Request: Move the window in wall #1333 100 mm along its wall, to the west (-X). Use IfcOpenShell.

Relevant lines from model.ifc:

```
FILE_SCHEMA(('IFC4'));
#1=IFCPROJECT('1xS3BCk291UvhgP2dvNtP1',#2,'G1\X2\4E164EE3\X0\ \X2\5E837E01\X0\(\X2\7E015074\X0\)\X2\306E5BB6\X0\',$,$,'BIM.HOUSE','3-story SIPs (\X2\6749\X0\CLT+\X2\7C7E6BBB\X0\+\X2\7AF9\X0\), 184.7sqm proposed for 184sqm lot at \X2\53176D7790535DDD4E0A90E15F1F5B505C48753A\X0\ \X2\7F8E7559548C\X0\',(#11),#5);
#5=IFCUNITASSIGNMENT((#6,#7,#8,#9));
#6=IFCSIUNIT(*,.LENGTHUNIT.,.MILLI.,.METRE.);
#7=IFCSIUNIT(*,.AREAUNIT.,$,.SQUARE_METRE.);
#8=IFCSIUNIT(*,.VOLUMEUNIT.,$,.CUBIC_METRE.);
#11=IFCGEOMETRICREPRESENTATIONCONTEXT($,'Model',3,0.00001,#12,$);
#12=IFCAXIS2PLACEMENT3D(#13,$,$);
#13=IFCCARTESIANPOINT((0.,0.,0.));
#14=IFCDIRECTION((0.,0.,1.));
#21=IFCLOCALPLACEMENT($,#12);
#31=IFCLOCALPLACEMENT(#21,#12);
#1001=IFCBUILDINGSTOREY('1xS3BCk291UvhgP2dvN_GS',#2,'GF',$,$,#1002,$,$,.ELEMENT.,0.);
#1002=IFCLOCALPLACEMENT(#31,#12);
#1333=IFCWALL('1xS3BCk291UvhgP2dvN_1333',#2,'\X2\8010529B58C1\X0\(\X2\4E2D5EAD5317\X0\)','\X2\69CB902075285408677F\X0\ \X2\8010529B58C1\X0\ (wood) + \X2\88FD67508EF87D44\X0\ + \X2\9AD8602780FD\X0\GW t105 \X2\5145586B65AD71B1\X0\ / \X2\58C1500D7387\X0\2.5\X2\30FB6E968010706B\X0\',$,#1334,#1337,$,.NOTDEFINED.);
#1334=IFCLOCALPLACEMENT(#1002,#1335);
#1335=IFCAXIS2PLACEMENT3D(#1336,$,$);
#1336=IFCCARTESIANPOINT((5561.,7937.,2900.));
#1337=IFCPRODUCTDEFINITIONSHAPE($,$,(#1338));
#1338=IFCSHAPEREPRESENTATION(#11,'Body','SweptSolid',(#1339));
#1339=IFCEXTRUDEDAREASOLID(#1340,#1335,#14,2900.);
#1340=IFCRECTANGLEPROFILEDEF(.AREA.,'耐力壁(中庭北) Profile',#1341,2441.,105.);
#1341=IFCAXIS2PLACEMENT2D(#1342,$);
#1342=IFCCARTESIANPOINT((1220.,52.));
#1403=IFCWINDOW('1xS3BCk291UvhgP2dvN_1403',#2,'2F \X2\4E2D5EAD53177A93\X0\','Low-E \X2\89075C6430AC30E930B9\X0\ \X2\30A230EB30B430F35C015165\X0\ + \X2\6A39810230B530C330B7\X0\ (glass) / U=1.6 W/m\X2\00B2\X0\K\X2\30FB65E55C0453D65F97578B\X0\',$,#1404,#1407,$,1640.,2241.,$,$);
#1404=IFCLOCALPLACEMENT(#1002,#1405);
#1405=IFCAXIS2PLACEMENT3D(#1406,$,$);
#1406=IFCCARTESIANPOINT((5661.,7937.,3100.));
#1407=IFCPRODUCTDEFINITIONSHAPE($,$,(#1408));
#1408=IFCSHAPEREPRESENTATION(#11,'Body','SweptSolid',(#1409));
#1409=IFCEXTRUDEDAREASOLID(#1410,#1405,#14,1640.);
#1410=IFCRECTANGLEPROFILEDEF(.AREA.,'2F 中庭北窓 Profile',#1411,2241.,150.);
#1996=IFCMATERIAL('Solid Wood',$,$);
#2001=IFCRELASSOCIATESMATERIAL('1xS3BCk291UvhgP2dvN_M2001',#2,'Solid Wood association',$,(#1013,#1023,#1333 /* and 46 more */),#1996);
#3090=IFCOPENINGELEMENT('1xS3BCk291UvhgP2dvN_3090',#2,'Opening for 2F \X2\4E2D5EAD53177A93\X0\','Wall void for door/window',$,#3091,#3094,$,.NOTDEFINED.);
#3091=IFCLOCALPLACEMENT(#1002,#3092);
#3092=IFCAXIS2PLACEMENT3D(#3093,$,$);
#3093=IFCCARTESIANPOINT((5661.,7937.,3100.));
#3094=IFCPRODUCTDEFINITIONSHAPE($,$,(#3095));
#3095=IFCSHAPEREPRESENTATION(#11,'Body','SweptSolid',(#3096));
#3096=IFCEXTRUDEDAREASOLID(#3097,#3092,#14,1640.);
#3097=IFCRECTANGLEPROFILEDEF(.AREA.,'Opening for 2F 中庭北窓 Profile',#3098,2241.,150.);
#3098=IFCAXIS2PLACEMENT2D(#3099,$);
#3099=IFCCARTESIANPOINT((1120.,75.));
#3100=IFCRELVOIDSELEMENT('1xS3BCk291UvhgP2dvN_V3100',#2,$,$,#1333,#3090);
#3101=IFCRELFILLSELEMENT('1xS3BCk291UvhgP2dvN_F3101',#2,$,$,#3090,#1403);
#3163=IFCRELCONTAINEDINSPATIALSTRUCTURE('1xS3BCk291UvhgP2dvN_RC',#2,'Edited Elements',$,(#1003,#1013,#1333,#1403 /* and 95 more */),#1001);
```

```python
import ifcopenshell
import ifcopenshell.api.geometry
import ifcopenshell.util.placement
import ifcopenshell.util.unit

model = ifcopenshell.open("model.ifc")
unit_scale = ifcopenshell.util.unit.calculate_unit_scale(model)

window = model.by_guid("1xS3BCk291UvhgP2dvN_1403")
opening = window.FillsVoids[0].RelatingOpeningElement
wall = opening.VoidsElements[0].RelatingBuildingElement

wall_matrix = ifcopenshell.util.placement.get_local_placement(wall.ObjectPlacement)
shift = wall_matrix[:3, 0] * -0.1 / unit_scale
before = ifcopenshell.util.placement.get_local_placement(window.ObjectPlacement)[:3, 3].copy()

# The window is not placed relative to its opening, so move both.
for product in (opening, window):
    matrix = ifcopenshell.util.placement.get_local_placement(product.ObjectPlacement)
    matrix[:3, 3] += shift
    ifcopenshell.api.geometry.edit_object_placement(model, product=product, matrix=matrix, is_si=False)

after = ifcopenshell.util.placement.get_local_placement(window.ObjectPlacement)[:3, 3]
print("window moved by", (after - before).round(3) + 0.0)

model.write("model_rev.ifc")
```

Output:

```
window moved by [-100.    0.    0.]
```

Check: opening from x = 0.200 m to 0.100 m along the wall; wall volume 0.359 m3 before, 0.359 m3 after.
